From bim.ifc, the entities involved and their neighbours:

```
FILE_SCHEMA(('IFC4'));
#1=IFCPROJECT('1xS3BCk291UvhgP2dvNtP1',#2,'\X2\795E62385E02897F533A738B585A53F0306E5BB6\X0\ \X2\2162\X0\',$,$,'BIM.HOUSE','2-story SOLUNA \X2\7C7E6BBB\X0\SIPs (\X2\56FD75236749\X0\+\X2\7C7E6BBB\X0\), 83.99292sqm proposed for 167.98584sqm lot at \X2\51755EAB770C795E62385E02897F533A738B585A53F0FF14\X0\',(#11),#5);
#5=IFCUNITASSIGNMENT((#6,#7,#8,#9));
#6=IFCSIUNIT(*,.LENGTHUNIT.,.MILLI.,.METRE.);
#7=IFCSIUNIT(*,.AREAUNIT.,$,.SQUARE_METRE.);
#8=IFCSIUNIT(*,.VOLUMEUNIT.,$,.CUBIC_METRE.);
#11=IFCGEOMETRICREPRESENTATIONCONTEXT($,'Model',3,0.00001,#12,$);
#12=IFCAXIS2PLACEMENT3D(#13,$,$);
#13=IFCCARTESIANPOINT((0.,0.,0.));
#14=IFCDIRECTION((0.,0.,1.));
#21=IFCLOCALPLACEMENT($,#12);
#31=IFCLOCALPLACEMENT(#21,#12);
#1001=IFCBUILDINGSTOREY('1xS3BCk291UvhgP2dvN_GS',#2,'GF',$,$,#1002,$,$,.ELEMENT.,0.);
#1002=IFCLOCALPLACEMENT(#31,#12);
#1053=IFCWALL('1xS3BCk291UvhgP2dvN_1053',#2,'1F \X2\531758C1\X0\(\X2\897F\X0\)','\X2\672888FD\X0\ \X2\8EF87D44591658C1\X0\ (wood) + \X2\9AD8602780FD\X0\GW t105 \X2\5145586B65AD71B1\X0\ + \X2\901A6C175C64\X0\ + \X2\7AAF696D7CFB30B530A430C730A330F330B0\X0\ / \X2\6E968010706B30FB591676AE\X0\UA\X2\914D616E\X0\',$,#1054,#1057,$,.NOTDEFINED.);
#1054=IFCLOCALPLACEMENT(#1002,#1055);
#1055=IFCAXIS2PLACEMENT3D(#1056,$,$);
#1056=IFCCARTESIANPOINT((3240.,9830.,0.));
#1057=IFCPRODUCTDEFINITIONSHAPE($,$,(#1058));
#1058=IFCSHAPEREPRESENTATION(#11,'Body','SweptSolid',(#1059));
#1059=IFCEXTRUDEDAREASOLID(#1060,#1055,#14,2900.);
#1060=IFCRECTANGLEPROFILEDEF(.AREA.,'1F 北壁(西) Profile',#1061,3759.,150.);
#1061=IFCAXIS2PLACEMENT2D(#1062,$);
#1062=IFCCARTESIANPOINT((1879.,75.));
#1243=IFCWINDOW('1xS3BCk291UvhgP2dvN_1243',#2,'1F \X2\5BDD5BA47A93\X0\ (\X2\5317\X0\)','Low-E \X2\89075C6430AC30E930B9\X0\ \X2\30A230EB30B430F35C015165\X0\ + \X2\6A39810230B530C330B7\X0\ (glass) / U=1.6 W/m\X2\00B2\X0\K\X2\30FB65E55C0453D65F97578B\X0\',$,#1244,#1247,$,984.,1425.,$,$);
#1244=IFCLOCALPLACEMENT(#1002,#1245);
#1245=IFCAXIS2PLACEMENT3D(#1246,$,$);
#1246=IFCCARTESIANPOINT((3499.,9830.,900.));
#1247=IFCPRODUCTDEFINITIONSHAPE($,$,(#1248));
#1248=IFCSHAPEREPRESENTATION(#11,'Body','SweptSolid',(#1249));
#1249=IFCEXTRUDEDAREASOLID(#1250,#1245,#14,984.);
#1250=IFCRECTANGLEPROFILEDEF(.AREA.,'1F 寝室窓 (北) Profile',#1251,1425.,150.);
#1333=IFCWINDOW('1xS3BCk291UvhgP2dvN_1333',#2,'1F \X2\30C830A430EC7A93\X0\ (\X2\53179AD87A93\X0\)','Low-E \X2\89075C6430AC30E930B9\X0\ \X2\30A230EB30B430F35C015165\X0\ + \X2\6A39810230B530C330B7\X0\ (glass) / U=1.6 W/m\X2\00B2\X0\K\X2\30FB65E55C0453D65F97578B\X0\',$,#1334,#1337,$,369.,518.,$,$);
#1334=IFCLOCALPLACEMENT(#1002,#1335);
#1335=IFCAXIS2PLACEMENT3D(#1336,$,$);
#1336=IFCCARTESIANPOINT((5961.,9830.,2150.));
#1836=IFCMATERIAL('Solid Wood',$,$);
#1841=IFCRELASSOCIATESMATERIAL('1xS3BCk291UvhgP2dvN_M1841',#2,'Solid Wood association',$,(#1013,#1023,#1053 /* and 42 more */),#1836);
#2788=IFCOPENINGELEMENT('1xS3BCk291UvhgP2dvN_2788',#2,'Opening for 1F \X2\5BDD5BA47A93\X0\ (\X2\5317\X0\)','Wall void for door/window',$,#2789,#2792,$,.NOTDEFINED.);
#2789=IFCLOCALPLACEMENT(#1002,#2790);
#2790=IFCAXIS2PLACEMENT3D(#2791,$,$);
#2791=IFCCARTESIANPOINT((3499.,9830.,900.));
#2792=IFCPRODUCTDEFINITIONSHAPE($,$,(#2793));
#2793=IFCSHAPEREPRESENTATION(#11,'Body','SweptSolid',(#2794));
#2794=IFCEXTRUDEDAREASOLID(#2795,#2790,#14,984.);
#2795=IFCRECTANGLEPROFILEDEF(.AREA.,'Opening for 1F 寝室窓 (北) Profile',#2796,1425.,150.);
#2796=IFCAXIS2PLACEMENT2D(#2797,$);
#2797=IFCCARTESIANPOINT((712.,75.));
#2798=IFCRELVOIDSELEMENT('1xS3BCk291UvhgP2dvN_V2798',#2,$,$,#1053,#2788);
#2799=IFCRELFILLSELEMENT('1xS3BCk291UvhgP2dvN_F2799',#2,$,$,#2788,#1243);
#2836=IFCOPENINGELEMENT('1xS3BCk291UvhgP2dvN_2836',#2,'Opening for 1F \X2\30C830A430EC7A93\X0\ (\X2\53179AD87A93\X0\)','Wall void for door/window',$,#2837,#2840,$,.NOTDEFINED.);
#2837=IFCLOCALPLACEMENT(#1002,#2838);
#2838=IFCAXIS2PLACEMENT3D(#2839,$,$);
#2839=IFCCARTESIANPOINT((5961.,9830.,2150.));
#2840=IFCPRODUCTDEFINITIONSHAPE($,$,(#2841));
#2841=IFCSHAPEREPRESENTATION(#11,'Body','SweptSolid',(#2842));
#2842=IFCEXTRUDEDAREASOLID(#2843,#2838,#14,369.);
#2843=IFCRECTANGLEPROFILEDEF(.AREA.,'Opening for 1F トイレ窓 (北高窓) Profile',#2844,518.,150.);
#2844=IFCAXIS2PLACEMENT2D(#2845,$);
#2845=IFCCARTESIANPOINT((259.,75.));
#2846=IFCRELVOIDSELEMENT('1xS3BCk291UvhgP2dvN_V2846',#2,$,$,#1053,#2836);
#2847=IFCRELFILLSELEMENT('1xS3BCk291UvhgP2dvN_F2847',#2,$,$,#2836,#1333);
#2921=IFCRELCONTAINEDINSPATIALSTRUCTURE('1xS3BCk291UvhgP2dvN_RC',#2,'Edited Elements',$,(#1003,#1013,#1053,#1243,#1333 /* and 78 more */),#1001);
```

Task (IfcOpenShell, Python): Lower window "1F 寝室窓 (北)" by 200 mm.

```python
import numpy as np
import ifcopenshell
import ifcopenshell.api.geometry
import ifcopenshell.util.placement
import ifcopenshell.util.unit

model = ifcopenshell.open("bim.ifc")
unit_scale = ifcopenshell.util.unit.calculate_unit_scale(model)

window = model.by_id(1243)
opening = window.FillsVoids[0].RelatingOpeningElement
dz = -0.2 / unit_scale

shift = np.array([0.0, 0.0, dz])
# The window is not placed relative to its opening, so move both.
for product in (opening, window):
    matrix = ifcopenshell.util.placement.get_local_placement(product.ObjectPlacement)
    matrix[:3, 3] += shift
    ifcopenshell.api.geometry.edit_object_placement(model, product=product, matrix=matrix, is_si=False)

print(f"moved by {dz * unit_scale:+.3f} m")

model.write("bim_updated.ifc")
```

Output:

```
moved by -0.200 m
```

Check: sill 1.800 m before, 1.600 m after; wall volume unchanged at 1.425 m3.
